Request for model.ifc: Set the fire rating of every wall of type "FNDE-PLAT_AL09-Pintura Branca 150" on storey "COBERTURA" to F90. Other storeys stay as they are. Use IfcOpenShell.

First a look at what the model holds.

```python
import ifcopenshell
import ifcopenshell.util.element

model = ifcopenshell.open("model.ifc")
print(model.schema)
storey = next(s for s in model.by_type("IfcBuildingStorey") if s.Name == "COBERTURA")
walls = [e for e in ifcopenshell.util.element.get_decomposition(storey) if e.is_a("IfcWall")]
seen = {}
for e in walls:
    element_type = ifcopenshell.util.element.get_type(e)
    key = (element_type.Name if element_type != e and element_type else None, ifcopenshell.util.element.get_pset(e, "Pset_WallCommon", "FireRating"))
    seen[key] = seen.get(key, 0) + 1
for (name, value), count in sorted(seen.items(), key=str):
    print(count, "x", name, "|", value)
```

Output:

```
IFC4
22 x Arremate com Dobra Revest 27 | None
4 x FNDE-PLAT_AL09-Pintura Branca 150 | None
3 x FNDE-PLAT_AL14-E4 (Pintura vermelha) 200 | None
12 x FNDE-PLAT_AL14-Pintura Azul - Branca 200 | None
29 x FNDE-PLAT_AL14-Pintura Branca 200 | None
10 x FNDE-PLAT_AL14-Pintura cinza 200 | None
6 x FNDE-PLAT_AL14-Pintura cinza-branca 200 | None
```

```python
import ifcopenshell
import ifcopenshell.api.pset
import ifcopenshell.util.element

model = ifcopenshell.open("model.ifc")

storey = next(s for s in model.by_type("IfcBuildingStorey") if s.Name == "COBERTURA")
walls = [e for e in ifcopenshell.util.element.get_decomposition(storey) if e.is_a("IfcWall")]

count = 0
for e in walls:
    element_type = ifcopenshell.util.element.get_type(e)
    if element_type in (None, e) or element_type.Name != "FNDE-PLAT_AL09-Pintura Branca 150":
        continue
    # add_pset returns the element's existing set when there is one.
    pset = ifcopenshell.api.pset.add_pset(model, product=e, name="Pset_WallCommon")
    ifcopenshell.api.pset.edit_pset(model, pset=pset, properties={"FireRating": "F90"})
    count += 1

print(count, "walls updated")

model.write("model-out.ifc")
```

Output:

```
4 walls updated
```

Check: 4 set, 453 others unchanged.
